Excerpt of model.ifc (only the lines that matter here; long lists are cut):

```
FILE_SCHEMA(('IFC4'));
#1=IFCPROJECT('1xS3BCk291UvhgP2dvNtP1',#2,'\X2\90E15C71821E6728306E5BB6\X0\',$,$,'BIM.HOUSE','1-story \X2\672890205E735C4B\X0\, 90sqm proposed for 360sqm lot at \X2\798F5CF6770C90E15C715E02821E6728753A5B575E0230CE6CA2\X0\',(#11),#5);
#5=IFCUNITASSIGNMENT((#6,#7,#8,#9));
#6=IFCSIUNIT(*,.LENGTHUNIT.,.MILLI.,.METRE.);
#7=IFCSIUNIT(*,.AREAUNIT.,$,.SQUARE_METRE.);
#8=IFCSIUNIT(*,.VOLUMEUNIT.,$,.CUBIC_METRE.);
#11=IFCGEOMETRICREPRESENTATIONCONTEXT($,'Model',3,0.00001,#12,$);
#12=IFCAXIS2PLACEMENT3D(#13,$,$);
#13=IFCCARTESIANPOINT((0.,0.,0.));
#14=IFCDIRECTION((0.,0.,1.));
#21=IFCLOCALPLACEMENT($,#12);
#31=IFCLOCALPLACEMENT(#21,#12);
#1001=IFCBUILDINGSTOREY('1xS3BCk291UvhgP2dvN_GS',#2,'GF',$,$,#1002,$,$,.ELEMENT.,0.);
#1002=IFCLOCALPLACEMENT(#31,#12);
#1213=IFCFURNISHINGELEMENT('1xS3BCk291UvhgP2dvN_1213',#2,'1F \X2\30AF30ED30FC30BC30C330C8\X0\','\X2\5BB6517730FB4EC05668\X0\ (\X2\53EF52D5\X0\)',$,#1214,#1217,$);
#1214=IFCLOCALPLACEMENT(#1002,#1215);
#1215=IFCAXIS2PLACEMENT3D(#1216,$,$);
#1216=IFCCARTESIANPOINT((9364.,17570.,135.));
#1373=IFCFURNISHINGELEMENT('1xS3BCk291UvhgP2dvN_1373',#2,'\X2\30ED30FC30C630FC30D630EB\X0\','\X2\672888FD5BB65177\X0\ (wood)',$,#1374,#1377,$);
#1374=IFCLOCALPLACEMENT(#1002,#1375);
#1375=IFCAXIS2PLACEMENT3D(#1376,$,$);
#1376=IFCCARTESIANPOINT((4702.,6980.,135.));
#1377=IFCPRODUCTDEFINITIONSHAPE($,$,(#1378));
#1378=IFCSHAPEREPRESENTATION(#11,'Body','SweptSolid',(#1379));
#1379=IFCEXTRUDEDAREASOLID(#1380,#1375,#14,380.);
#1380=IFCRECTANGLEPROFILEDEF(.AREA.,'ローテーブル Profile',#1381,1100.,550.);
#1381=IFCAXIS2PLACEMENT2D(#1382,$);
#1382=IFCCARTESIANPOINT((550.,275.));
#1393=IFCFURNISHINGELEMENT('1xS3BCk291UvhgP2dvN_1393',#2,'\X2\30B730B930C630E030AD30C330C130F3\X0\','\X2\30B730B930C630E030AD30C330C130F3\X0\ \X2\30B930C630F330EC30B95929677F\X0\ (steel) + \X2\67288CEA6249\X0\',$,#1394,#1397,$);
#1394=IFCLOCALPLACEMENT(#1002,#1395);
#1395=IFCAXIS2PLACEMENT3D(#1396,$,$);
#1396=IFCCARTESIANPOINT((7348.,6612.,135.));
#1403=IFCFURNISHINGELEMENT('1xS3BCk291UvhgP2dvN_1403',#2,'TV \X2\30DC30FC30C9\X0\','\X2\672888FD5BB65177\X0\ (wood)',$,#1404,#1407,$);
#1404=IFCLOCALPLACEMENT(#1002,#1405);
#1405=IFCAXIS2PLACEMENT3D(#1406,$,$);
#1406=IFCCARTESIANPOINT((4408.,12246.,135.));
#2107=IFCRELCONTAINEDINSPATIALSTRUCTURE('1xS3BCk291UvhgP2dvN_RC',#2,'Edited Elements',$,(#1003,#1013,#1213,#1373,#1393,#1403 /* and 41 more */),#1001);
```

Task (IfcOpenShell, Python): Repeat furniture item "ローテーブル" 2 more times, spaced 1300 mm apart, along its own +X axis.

```python
import ifcopenshell
import ifcopenshell.api.geometry
import ifcopenshell.api.root
import ifcopenshell.util.element
import ifcopenshell.util.placement
import ifcopenshell.util.unit

model = ifcopenshell.open("model.ifc")
unit_scale = ifcopenshell.util.unit.calculate_unit_scale(model)


def reuse_history(source, copy):
    """copy_class also copies each property set's owner history, people and application; keep the originals."""
    for rel in copy.IsDefinedBy:
        if rel.is_a("IfcRelDefinesByProperties") and (history := rel.RelatingPropertyDefinition.OwnerHistory):
            rel.RelatingPropertyDefinition.OwnerHistory = source.OwnerHistory
            ifcopenshell.util.element.remove_deep2(model, history)


source = model.by_guid("1xS3BCk291UvhgP2dvN_1373")
base = ifcopenshell.util.placement.get_local_placement(source.ObjectPlacement)
step = base[:3, 0] * 1.3 / unit_scale

for i in range(1, 3):
    copy = ifcopenshell.api.root.copy_class(model, product=source)
    copy.Representation = ifcopenshell.util.element.copy_deep(
        model, source.Representation, exclude=["IfcGeometricRepresentationContext", "IfcRepresentationMap"]
    )
    reuse_history(source, copy)
    matrix = base.copy()
    matrix[:3, 3] += i * step
    print("added at", matrix[:3, 3].round(3) + 0.0)
    ifcopenshell.api.geometry.edit_object_placement(model, product=copy, matrix=matrix, is_si=False)

model.write("model_rev.ifc")
```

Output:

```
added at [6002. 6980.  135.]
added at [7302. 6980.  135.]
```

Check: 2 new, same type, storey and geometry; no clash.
